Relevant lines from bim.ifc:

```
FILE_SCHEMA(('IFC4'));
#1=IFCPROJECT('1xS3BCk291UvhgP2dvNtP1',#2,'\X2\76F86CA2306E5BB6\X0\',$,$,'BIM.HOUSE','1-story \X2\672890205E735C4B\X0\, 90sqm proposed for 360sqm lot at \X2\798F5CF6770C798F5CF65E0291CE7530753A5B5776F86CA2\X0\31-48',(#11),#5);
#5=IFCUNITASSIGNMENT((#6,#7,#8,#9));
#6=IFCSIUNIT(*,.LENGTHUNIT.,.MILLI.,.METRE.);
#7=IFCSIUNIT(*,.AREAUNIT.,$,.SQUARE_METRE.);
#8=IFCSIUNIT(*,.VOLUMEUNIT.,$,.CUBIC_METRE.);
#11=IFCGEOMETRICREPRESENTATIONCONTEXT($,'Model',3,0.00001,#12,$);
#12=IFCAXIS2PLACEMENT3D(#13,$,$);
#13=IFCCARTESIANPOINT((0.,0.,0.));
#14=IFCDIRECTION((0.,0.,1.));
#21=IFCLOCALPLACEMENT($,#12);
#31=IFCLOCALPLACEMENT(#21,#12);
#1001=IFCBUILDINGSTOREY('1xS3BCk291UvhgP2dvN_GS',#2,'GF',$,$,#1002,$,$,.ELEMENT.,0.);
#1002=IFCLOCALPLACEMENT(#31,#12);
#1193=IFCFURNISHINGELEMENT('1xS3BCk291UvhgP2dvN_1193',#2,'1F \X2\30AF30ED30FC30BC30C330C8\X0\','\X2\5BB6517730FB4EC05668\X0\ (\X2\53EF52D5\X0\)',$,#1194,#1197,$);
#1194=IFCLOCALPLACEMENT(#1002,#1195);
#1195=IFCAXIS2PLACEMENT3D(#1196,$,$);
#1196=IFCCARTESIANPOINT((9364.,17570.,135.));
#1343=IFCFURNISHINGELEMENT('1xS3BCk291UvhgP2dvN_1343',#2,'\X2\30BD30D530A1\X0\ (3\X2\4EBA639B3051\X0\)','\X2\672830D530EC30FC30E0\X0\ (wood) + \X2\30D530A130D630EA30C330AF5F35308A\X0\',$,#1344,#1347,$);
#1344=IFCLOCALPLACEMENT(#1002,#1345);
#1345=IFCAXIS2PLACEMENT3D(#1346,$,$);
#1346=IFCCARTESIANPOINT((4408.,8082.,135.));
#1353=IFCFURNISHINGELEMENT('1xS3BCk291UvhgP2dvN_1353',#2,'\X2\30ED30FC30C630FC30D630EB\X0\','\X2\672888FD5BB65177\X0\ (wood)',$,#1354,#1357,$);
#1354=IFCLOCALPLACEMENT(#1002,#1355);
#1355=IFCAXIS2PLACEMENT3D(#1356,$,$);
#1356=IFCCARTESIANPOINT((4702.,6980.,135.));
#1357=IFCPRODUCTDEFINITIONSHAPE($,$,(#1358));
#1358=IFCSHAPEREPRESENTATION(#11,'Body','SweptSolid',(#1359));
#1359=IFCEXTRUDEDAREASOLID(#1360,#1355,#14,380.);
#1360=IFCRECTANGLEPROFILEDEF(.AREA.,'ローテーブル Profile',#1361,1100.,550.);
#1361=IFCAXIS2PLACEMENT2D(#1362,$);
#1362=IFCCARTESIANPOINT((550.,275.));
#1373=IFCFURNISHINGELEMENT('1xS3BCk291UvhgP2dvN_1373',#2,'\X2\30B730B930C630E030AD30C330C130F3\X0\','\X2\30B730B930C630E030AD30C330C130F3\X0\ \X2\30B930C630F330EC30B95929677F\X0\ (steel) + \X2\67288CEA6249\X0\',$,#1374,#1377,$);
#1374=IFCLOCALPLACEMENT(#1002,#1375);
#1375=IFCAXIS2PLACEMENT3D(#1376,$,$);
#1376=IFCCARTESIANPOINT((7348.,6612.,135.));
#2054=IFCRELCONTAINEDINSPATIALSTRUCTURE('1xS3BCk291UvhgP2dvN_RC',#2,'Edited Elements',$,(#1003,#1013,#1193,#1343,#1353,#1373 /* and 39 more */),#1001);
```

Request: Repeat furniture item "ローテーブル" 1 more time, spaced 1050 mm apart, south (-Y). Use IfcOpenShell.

```python
import numpy as np
import ifcopenshell
import ifcopenshell.api.geometry
import ifcopenshell.api.root
import ifcopenshell.util.element
import ifcopenshell.util.placement
import ifcopenshell.util.unit

model = ifcopenshell.open("bim.ifc")
unit_scale = ifcopenshell.util.unit.calculate_unit_scale(model)


def reuse_history(source, copy):
    """copy_class also copies each property set's owner history, people and application; keep the originals."""
    for rel in copy.IsDefinedBy:
        if rel.is_a("IfcRelDefinesByProperties") and (history := rel.RelatingPropertyDefinition.OwnerHistory):
            rel.RelatingPropertyDefinition.OwnerHistory = source.OwnerHistory
            ifcopenshell.util.element.remove_deep2(model, history)


source = model.by_guid("1xS3BCk291UvhgP2dvN_1353")
base = ifcopenshell.util.placement.get_local_placement(source.ObjectPlacement)
step = np.array([0.0, -1.0, 0.0]) * 1.05 / unit_scale

for i in range(1, 2):
    copy = ifcopenshell.api.root.copy_class(model, product=source)
    copy.Representation = ifcopenshell.util.element.copy_deep(
        model, source.Representation, exclude=["IfcGeometricRepresentationContext", "IfcRepresentationMap"]
    )
    reuse_history(source, copy)
    matrix = base.copy()
    matrix[:3, 3] += i * step
    print("added at", matrix[:3, 3].round(3) + 0.0)
    ifcopenshell.api.geometry.edit_object_placement(model, product=copy, matrix=matrix, is_si=False)

model.write("bim-out.ifc")
```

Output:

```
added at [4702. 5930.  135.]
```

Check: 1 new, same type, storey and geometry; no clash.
